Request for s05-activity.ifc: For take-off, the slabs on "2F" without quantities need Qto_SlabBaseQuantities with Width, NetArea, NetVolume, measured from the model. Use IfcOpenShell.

First a look at what the model holds.

```python
import ifcopenshell
import ifcopenshell.util.element
import ifcopenshell.util.unit

model = ifcopenshell.open("s05-activity.ifc")
print(model.schema)
for unit_type in ("LENGTHUNIT", "AREAUNIT", "VOLUMEUNIT"):
    print(unit_type, ifcopenshell.util.unit.calculate_unit_scale(model, unit_type))
storey = next(s for s in model.by_type("IfcBuildingStorey") if s.Name == "2F")
slabs = [e for e in ifcopenshell.util.element.get_decomposition(storey) if e.is_a("IfcSlab")]
for e in sorted(slabs, key=lambda e: e.id()):
    print(e.id(), e.is_a(), e.Name, list(ifcopenshell.util.element.get_psets(e, qtos_only=True)), sep=" | ")
```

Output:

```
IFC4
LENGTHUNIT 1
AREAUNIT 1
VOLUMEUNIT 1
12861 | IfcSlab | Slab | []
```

```python
import ifcopenshell
import ifcopenshell.api.pset
import ifcopenshell.geom
import ifcopenshell.util.element
import ifcopenshell.util.shape
import ifcopenshell.util.unit

model = ifcopenshell.open("s05-activity.ifc")
unit_scale = ifcopenshell.util.unit.calculate_unit_scale(model)
area_scale = ifcopenshell.util.unit.calculate_unit_scale(model, "AREAUNIT")
volume_scale = ifcopenshell.util.unit.calculate_unit_scale(model, "VOLUMEUNIT")
settings = ifcopenshell.geom.settings()

storey = next(s for s in model.by_type("IfcBuildingStorey") if s.Name == "2F")
slabs = [e for e in ifcopenshell.util.element.get_decomposition(storey) if e.is_a("IfcSlab")]

for e in sorted(slabs, key=lambda e: e.id()):
    if ifcopenshell.util.element.get_psets(e, qtos_only=True, should_inherit=False):
        continue
    # Geometry comes back in metres, in the element's own axes.
    shape = ifcopenshell.geom.create_shape(settings, e)
    values = {
        "Width": ifcopenshell.util.shape.get_z(shape.geometry) / unit_scale,
        "NetArea": ifcopenshell.util.shape.get_footprint_area(shape.geometry) / area_scale,
        "NetVolume": ifcopenshell.util.shape.get_volume(shape.geometry) / volume_scale,
    }
    qto = ifcopenshell.api.pset.add_qto(model, product=e, name="Qto_SlabBaseQuantities")
    ifcopenshell.api.pset.edit_qto(model, qto=qto, properties=values)
    print(e.id(), {k: round(v, 3) for k, v in values.items()})

model.write("s05-activity_rev.ifc")
```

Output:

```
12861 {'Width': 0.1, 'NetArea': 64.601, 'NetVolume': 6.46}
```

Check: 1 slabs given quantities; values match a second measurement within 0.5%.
